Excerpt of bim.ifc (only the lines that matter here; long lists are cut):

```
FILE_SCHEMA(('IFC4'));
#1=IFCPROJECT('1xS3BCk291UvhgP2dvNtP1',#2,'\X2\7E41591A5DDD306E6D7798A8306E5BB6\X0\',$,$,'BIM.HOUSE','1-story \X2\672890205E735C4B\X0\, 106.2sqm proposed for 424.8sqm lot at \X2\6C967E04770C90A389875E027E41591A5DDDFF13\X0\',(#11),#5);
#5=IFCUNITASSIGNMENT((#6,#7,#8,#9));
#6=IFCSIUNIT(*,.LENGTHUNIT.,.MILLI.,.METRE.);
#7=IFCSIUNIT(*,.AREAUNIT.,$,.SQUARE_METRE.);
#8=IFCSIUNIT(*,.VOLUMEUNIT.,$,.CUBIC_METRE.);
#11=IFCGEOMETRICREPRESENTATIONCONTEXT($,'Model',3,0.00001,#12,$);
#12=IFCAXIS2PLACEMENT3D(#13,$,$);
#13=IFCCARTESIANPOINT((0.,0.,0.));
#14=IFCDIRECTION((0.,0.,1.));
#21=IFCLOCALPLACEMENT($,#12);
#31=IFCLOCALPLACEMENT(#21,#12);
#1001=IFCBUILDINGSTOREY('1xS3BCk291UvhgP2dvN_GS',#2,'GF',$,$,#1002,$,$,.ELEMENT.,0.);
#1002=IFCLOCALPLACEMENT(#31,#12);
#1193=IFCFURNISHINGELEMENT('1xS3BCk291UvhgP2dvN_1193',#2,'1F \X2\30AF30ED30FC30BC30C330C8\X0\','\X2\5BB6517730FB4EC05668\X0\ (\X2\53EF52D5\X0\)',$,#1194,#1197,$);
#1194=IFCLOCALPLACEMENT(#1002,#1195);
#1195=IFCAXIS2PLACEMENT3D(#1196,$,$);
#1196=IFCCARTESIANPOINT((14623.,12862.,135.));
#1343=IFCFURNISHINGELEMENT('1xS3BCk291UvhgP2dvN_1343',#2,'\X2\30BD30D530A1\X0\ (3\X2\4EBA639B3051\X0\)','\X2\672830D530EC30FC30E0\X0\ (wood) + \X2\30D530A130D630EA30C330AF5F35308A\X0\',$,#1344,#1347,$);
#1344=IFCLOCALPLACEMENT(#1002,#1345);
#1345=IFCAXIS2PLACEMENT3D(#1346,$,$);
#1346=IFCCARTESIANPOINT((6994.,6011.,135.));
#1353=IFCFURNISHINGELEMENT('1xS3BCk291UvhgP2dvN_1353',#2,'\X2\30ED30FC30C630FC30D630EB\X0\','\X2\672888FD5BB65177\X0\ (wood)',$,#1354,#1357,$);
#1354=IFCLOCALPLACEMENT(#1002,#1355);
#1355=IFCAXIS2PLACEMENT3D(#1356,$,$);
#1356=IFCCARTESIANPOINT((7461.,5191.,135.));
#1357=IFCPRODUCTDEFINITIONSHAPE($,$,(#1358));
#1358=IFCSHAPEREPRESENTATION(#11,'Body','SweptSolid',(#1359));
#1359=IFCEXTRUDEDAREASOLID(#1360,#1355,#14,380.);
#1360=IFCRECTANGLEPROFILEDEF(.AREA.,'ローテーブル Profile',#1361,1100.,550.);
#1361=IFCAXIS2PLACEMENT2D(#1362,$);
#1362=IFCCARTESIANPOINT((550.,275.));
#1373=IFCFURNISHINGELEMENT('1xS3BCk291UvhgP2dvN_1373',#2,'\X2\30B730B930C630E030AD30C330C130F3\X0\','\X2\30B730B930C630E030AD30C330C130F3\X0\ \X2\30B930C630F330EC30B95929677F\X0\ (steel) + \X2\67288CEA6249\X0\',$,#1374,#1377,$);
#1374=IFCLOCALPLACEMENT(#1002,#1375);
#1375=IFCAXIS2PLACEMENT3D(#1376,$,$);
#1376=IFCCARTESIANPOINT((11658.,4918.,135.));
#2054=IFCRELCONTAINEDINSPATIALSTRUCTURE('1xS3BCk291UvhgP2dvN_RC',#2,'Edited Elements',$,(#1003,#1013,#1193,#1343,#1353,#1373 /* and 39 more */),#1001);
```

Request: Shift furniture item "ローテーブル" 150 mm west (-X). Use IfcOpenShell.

```python
import ifcopenshell
import ifcopenshell.api.geometry
import ifcopenshell.util.placement

model = ifcopenshell.open("bim.ifc")

item = model.by_id(1353)
matrix = ifcopenshell.util.placement.get_local_placement(item.ObjectPlacement)
matrix[0, 3] -= 150.0
ifcopenshell.api.geometry.edit_object_placement(model, product=item, matrix=matrix, is_si=False)

print(ifcopenshell.util.placement.get_local_placement(item.ObjectPlacement).round(3) + 0.0)

model.write("bim_edited.ifc")
```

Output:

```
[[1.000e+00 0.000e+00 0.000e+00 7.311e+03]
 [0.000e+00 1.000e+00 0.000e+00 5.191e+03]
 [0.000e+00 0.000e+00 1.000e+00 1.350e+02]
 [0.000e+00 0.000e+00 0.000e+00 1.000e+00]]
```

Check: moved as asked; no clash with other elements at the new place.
